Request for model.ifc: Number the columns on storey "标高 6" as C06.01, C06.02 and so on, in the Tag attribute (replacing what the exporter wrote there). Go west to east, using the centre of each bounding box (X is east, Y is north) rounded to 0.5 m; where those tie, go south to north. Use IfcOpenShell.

First a look at what the model holds.

```python
import ifcopenshell
import ifcopenshell.util.element
import ifcopenshell.util.placement

model = ifcopenshell.open("model.ifc")
print(model.schema)
storey = next(s for s in model.by_type("IfcBuildingStorey") if s.Name == "标高 6")
columns = [e for e in ifcopenshell.util.element.get_decomposition(storey) if e.is_a("IfcColumn")]
for e in sorted(columns, key=lambda e: e.id()):
    origin = ifcopenshell.util.placement.get_local_placement(e.ObjectPlacement)[:3, 3]
    print(e.id(), e.Tag, e.Name, origin.round(2) + 0.0, sep=" | ")
```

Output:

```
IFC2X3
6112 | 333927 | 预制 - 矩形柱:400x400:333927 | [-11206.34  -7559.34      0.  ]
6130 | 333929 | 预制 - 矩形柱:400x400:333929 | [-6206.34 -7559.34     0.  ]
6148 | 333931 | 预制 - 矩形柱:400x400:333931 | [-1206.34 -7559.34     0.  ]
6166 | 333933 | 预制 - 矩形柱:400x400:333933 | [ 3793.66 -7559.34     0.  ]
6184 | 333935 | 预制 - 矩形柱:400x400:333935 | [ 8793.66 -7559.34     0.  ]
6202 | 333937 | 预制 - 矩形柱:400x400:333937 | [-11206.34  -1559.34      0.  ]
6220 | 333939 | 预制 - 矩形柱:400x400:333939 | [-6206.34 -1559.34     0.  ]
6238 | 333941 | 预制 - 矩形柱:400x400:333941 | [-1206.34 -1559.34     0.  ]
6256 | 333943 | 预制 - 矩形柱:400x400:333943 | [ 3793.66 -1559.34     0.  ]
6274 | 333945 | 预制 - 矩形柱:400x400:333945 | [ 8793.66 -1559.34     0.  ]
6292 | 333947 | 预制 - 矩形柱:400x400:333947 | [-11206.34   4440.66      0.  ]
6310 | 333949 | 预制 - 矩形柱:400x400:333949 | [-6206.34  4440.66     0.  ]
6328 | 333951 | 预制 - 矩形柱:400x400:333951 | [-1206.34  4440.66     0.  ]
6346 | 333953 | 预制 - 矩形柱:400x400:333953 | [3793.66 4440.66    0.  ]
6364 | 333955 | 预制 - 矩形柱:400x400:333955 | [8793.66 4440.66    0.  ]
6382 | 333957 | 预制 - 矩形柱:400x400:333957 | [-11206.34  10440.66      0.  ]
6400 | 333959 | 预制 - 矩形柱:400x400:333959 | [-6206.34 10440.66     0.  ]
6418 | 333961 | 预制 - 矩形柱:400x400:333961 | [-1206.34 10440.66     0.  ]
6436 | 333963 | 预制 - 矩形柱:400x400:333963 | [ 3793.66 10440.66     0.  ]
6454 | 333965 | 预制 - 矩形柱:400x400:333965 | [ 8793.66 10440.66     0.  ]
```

```python
import ifcopenshell
import ifcopenshell.geom
import ifcopenshell.util.element
import ifcopenshell.util.shape

model = ifcopenshell.open("model.ifc")
settings = ifcopenshell.geom.settings()
settings.set("use-world-coords", True)


def centre(element):
    shape = ifcopenshell.geom.create_shape(settings, element)
    return ifcopenshell.util.shape.get_bbox_centroid(shape.geometry)


storey = next(s for s in model.by_type("IfcBuildingStorey") if s.Name == "标高 6")
columns = [e for e in ifcopenshell.util.element.get_decomposition(storey) if e.is_a("IfcColumn")]

# Insertion points can sit at a corner or the storey origin, so sort by the geometry (in metres).
centres = {e: centre(e) for e in columns}
columns.sort(key=lambda e: (round(centres[e][0] / 0.5), centres[e][1]))

for i, e in enumerate(columns, start=1):
    number = f"C06.{i:02d}"
    e.Tag = number
    print(e.id(), number)

model.write("model_rev.ifc")
```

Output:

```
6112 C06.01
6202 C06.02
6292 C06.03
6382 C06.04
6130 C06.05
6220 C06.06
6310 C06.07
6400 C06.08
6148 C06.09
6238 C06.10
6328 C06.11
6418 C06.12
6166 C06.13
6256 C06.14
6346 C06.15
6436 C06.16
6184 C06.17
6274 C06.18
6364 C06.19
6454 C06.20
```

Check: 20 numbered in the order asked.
